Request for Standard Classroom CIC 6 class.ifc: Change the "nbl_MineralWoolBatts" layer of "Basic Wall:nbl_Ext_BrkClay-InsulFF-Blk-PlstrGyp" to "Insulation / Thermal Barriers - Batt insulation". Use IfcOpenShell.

First a look at what the model holds.

```python
import ifcopenshell
import ifcopenshell.util.element

model = ifcopenshell.open("Standard Classroom CIC 6 class.ifc")
print(model.schema)
for layer_set in model.by_type("IfcMaterialLayerSet"):
    if layer_set.LayerSetName == "Basic Wall:nbl_Ext_BrkClay-InsulFF-Blk-PlstrGyp":
        for layer in layer_set.MaterialLayers:
            print(layer.id(), layer.Material and layer.Material.Name, layer.LayerThickness, sep=" | ")
        print(len(ifcopenshell.util.element.get_elements_by_material(model, layer_set)), "elements and types use it")
print(sorted(m.Name for m in model.by_type("IfcMaterial") if m.Name)[:60])
```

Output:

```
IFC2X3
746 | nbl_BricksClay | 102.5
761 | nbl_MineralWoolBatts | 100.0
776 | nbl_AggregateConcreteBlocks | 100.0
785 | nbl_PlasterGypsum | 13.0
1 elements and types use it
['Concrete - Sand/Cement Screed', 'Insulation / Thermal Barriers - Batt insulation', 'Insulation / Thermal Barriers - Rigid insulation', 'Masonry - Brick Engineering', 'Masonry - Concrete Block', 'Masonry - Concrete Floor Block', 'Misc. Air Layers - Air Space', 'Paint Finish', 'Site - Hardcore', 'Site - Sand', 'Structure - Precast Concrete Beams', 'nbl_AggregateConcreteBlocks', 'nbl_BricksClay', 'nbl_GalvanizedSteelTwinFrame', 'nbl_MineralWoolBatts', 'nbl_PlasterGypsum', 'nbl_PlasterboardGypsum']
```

```python
import ifcopenshell
import ifcopenshell.api.material

model = ifcopenshell.open("Standard Classroom CIC 6 class.ifc")

layer_set = next(s for s in model.by_type("IfcMaterialLayerSet") if s.LayerSetName == "Basic Wall:nbl_Ext_BrkClay-InsulFF-Blk-PlstrGyp")
layer = next(l for l in layer_set.MaterialLayers if l.Material and l.Material.Name == "nbl_MineralWoolBatts")
material = next(m for m in model.by_type("IfcMaterial") if m.Name == "Insulation / Thermal Barriers - Batt insulation")

# Point this one layer at the other material; renaming the old one would change it everywhere.
ifcopenshell.api.material.edit_layer(model, layer=layer, attributes={}, material=material)

print([l.Material.Name if l.Material else None for l in layer_set.MaterialLayers])

model.write("Standard Classroom CIC 6 class-out.ifc")
```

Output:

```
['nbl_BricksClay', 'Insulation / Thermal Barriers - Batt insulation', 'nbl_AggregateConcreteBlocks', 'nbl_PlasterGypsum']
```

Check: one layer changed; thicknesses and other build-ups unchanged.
